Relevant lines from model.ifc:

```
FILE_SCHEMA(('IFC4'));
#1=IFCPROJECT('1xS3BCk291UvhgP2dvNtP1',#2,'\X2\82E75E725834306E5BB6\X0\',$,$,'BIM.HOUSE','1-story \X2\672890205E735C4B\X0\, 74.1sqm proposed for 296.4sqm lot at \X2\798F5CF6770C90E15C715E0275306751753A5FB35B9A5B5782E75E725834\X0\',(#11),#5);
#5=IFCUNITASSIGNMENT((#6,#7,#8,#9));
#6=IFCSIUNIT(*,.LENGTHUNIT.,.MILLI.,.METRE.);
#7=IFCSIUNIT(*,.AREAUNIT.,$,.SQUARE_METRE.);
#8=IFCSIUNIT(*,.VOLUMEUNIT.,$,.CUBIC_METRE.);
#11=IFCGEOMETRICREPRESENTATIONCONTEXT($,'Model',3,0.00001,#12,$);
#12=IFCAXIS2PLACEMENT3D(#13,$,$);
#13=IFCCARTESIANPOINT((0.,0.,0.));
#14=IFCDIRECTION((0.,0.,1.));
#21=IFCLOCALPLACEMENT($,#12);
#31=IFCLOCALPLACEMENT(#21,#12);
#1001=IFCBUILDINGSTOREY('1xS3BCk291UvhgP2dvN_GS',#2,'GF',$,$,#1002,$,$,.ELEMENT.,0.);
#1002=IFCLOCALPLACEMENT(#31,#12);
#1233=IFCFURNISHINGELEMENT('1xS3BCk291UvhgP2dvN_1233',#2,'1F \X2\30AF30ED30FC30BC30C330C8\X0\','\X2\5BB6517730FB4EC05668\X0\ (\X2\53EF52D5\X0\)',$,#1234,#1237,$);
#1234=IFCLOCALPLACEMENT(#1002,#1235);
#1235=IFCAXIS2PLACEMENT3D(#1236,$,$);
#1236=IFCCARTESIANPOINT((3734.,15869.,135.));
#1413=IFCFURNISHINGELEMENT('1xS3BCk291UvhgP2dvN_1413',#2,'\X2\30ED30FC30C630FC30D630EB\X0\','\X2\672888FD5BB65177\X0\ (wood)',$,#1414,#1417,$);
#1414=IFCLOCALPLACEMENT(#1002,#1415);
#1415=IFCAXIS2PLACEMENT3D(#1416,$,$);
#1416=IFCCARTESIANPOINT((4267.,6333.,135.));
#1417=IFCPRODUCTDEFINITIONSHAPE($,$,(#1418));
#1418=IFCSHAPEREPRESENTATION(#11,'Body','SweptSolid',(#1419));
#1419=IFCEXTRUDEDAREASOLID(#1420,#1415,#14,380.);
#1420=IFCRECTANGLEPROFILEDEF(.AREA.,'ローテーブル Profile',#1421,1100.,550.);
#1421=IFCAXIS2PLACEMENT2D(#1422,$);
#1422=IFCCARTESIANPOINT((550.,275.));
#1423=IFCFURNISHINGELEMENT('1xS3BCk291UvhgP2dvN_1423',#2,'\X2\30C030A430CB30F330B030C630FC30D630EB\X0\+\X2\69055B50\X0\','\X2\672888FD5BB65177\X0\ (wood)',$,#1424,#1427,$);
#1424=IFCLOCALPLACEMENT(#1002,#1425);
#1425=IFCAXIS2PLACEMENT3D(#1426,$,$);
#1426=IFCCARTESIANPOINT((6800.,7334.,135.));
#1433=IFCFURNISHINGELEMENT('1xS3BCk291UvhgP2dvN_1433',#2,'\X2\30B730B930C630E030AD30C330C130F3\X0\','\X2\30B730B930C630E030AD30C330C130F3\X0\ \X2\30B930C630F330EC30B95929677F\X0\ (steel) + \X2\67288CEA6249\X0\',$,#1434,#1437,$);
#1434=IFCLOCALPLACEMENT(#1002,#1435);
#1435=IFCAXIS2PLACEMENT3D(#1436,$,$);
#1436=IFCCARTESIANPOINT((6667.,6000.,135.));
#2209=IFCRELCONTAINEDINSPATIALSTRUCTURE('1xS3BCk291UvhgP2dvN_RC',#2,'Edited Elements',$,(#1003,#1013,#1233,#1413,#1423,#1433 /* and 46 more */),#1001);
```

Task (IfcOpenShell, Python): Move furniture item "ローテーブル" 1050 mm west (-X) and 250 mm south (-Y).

```python
import ifcopenshell
import ifcopenshell.api.geometry
import ifcopenshell.util.placement
import ifcopenshell.util.unit

model = ifcopenshell.open("model.ifc")
unit_scale = ifcopenshell.util.unit.calculate_unit_scale(model)

item = model.by_guid("1xS3BCk291UvhgP2dvN_1413")
matrix = ifcopenshell.util.placement.get_local_placement(item.ObjectPlacement)
matrix[0, 3] -= 1.05 / unit_scale
matrix[1, 3] -= 0.25 / unit_scale
ifcopenshell.api.geometry.edit_object_placement(model, product=item, matrix=matrix, is_si=False)

print(ifcopenshell.util.placement.get_local_placement(item.ObjectPlacement).round(3) + 0.0)

model.write("model-out.ifc")
```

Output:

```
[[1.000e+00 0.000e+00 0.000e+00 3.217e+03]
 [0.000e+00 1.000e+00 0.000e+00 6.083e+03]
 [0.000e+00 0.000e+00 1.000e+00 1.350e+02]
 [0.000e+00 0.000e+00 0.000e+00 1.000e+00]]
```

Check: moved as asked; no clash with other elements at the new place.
